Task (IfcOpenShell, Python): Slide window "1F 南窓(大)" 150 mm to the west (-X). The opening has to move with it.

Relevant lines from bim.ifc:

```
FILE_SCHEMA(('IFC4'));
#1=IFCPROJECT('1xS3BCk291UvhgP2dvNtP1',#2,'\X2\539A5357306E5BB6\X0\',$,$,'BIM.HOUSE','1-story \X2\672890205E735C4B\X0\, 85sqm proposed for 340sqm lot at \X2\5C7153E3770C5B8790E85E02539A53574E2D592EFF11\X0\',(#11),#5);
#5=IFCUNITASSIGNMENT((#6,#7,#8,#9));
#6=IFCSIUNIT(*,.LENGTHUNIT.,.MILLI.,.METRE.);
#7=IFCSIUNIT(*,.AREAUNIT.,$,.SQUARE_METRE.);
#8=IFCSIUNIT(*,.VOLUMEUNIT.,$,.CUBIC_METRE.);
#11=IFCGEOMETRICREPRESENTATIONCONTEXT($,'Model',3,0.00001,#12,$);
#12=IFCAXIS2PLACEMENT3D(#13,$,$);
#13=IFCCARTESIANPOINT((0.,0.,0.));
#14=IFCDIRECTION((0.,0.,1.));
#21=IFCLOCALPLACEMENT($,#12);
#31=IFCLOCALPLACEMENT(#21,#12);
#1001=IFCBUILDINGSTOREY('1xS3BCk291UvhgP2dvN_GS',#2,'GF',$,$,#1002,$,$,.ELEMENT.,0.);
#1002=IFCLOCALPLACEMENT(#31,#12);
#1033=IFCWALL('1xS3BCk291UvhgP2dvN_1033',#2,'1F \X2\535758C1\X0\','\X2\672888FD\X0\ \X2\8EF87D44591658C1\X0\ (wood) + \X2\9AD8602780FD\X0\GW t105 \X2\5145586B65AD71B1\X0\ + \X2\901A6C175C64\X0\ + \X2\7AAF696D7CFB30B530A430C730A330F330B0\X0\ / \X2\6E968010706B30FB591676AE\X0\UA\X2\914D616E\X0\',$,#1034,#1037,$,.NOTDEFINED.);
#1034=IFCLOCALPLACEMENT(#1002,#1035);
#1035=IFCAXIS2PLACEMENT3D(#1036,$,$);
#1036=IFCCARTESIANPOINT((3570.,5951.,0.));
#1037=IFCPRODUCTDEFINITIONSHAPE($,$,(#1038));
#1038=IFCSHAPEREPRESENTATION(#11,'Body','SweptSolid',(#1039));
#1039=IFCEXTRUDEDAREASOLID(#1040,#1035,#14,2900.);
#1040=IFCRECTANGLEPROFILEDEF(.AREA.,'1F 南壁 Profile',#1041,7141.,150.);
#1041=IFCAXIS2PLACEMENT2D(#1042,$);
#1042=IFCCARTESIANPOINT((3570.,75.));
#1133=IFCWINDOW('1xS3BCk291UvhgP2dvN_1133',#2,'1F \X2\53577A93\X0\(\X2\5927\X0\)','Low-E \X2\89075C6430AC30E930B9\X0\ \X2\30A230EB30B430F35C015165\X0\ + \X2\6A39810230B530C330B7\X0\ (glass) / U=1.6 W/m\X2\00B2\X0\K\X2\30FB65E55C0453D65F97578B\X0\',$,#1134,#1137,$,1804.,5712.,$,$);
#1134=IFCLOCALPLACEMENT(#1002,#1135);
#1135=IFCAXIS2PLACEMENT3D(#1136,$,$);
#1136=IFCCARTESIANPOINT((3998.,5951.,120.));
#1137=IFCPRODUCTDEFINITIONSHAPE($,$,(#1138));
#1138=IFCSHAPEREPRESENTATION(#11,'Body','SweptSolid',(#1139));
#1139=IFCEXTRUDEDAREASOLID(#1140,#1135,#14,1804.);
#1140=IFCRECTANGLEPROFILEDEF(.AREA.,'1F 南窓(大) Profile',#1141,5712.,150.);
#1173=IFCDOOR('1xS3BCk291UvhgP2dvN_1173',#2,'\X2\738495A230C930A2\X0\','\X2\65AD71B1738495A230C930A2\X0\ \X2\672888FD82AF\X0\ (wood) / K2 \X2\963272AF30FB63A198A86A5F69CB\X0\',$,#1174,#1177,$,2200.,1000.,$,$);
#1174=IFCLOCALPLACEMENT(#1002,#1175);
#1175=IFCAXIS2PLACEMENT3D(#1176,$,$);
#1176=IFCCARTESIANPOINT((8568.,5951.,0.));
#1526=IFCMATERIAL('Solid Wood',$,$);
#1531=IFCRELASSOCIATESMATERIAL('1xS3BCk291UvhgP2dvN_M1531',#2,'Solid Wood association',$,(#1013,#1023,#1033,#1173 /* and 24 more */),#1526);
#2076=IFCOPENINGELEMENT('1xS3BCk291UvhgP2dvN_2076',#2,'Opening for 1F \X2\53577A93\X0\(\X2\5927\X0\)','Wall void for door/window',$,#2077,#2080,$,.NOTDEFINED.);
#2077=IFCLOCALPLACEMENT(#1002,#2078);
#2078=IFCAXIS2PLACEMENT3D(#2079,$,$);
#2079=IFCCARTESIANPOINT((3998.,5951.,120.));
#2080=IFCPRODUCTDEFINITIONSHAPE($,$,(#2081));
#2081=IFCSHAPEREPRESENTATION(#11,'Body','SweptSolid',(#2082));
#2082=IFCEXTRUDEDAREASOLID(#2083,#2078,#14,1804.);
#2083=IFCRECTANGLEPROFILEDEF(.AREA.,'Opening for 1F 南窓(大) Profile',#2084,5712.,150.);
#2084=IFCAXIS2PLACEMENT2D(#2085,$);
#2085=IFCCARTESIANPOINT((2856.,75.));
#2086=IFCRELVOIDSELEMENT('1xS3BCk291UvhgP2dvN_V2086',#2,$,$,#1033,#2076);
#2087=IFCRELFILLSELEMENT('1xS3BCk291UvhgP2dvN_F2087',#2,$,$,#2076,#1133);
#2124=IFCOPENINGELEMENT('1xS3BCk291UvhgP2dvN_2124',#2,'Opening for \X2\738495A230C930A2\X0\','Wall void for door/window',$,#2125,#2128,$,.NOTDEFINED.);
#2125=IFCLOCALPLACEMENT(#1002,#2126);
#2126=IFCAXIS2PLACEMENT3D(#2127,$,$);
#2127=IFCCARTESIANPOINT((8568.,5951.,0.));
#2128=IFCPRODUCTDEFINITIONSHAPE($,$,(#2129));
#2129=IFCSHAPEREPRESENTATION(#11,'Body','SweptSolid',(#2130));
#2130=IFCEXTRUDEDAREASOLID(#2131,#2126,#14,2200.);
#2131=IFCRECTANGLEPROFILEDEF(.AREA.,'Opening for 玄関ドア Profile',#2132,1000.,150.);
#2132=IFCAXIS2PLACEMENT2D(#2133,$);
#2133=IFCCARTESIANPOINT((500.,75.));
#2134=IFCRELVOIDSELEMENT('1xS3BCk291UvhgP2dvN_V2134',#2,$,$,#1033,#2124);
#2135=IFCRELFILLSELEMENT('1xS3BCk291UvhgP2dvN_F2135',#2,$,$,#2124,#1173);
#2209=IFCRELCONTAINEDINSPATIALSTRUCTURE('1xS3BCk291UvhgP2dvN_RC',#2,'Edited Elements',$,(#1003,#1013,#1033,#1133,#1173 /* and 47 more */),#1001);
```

```python
import ifcopenshell
import ifcopenshell.api.geometry
import ifcopenshell.util.placement
import ifcopenshell.util.unit

model = ifcopenshell.open("bim.ifc")
unit_scale = ifcopenshell.util.unit.calculate_unit_scale(model)

window = model.by_guid("1xS3BCk291UvhgP2dvN_1133")
opening = window.FillsVoids[0].RelatingOpeningElement
wall = opening.VoidsElements[0].RelatingBuildingElement

wall_matrix = ifcopenshell.util.placement.get_local_placement(wall.ObjectPlacement)
shift = wall_matrix[:3, 0] * -0.15 / unit_scale
before = ifcopenshell.util.placement.get_local_placement(window.ObjectPlacement)[:3, 3].copy()

# The window is not placed relative to its opening, so move both.
for product in (opening, window):
    matrix = ifcopenshell.util.placement.get_local_placement(product.ObjectPlacement)
    matrix[:3, 3] += shift
    ifcopenshell.api.geometry.edit_object_placement(model, product=product, matrix=matrix, is_si=False)

after = ifcopenshell.util.placement.get_local_placement(window.ObjectPlacement)[:3, 3]
print("window moved by", (after - before).round(3) + 0.0)

model.write("bim_updated.ifc")
```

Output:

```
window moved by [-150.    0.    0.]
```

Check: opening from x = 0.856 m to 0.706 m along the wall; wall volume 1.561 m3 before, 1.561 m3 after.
